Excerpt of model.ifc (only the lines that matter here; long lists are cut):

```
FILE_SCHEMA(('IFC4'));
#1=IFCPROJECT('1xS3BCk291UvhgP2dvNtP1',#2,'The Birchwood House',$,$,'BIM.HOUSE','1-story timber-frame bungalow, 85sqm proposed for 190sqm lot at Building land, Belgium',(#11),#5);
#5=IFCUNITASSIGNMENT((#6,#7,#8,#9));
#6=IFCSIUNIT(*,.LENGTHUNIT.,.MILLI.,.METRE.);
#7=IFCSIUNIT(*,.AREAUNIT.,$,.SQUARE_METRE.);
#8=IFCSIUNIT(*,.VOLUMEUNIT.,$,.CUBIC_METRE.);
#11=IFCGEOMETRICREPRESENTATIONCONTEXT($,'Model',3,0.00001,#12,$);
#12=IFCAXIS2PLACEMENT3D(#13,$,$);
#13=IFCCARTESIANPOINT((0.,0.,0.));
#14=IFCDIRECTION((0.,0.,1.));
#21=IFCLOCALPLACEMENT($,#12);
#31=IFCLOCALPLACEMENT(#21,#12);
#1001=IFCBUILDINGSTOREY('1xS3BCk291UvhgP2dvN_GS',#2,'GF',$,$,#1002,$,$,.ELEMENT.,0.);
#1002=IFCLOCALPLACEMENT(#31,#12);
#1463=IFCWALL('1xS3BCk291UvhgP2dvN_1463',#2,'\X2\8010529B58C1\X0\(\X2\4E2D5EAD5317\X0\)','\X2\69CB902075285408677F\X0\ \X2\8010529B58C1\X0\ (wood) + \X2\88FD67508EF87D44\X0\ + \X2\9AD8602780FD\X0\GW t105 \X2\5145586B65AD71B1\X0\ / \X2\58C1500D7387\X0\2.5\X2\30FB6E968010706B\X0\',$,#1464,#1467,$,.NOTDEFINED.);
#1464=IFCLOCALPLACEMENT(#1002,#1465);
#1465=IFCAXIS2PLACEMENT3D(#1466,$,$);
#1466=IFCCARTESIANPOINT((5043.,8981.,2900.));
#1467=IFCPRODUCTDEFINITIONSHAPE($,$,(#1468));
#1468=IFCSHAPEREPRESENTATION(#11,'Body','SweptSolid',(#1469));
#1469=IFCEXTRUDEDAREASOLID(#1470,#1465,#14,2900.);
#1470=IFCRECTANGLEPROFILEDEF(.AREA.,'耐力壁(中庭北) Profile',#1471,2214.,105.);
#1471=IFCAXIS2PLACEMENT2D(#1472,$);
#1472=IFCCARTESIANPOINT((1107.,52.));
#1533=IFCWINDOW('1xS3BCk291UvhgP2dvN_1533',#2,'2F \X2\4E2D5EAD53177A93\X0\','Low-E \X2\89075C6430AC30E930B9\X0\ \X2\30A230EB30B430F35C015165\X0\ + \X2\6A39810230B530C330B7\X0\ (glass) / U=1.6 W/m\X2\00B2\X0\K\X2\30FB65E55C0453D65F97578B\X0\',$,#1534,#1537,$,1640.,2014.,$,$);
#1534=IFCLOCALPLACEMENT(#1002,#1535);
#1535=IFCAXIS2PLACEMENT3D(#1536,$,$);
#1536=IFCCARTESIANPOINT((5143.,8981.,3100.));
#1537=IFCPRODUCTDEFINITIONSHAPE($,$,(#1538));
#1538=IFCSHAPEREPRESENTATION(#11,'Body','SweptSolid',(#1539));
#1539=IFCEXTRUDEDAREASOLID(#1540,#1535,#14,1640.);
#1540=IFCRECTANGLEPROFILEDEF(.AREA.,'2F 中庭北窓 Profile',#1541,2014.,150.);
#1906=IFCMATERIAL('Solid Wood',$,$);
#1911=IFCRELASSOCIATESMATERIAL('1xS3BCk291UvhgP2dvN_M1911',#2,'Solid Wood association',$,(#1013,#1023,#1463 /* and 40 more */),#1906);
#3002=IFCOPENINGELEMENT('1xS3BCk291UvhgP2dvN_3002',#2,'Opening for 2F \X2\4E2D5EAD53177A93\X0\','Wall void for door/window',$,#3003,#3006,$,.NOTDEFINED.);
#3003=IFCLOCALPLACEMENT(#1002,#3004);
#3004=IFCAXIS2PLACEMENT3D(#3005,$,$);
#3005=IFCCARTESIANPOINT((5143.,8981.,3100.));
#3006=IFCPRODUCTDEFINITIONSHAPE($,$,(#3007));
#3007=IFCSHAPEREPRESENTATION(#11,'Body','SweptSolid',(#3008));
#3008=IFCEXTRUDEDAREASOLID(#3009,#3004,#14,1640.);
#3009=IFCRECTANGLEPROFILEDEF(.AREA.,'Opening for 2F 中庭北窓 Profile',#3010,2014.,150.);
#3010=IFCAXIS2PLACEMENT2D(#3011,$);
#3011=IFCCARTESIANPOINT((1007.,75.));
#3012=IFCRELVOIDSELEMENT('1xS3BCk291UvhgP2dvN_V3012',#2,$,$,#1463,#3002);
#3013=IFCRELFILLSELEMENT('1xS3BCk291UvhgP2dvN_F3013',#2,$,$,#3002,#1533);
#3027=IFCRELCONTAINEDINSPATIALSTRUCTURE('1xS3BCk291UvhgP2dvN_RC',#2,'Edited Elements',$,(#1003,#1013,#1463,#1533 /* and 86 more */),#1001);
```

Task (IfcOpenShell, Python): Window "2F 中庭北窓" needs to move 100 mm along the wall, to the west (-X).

```python
import ifcopenshell
import ifcopenshell.api.geometry
import ifcopenshell.util.placement

model = ifcopenshell.open("model.ifc")

window = model.by_id(1533)
opening = window.FillsVoids[0].RelatingOpeningElement
wall = opening.VoidsElements[0].RelatingBuildingElement

wall_matrix = ifcopenshell.util.placement.get_local_placement(wall.ObjectPlacement)
shift = wall_matrix[:3, 0] * -100.0
before = ifcopenshell.util.placement.get_local_placement(window.ObjectPlacement)[:3, 3].copy()

# The window is not placed relative to its opening, so move both.
for product in (opening, window):
    matrix = ifcopenshell.util.placement.get_local_placement(product.ObjectPlacement)
    matrix[:3, 3] += shift
    ifcopenshell.api.geometry.edit_object_placement(model, product=product, matrix=matrix, is_si=False)

after = ifcopenshell.util.placement.get_local_placement(window.ObjectPlacement)[:3, 3]
print("window moved by", (after - before).round(3) + 0.0)

model.write("model_rev.ifc")
```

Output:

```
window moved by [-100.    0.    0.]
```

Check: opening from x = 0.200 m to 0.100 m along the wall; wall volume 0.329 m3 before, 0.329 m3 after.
